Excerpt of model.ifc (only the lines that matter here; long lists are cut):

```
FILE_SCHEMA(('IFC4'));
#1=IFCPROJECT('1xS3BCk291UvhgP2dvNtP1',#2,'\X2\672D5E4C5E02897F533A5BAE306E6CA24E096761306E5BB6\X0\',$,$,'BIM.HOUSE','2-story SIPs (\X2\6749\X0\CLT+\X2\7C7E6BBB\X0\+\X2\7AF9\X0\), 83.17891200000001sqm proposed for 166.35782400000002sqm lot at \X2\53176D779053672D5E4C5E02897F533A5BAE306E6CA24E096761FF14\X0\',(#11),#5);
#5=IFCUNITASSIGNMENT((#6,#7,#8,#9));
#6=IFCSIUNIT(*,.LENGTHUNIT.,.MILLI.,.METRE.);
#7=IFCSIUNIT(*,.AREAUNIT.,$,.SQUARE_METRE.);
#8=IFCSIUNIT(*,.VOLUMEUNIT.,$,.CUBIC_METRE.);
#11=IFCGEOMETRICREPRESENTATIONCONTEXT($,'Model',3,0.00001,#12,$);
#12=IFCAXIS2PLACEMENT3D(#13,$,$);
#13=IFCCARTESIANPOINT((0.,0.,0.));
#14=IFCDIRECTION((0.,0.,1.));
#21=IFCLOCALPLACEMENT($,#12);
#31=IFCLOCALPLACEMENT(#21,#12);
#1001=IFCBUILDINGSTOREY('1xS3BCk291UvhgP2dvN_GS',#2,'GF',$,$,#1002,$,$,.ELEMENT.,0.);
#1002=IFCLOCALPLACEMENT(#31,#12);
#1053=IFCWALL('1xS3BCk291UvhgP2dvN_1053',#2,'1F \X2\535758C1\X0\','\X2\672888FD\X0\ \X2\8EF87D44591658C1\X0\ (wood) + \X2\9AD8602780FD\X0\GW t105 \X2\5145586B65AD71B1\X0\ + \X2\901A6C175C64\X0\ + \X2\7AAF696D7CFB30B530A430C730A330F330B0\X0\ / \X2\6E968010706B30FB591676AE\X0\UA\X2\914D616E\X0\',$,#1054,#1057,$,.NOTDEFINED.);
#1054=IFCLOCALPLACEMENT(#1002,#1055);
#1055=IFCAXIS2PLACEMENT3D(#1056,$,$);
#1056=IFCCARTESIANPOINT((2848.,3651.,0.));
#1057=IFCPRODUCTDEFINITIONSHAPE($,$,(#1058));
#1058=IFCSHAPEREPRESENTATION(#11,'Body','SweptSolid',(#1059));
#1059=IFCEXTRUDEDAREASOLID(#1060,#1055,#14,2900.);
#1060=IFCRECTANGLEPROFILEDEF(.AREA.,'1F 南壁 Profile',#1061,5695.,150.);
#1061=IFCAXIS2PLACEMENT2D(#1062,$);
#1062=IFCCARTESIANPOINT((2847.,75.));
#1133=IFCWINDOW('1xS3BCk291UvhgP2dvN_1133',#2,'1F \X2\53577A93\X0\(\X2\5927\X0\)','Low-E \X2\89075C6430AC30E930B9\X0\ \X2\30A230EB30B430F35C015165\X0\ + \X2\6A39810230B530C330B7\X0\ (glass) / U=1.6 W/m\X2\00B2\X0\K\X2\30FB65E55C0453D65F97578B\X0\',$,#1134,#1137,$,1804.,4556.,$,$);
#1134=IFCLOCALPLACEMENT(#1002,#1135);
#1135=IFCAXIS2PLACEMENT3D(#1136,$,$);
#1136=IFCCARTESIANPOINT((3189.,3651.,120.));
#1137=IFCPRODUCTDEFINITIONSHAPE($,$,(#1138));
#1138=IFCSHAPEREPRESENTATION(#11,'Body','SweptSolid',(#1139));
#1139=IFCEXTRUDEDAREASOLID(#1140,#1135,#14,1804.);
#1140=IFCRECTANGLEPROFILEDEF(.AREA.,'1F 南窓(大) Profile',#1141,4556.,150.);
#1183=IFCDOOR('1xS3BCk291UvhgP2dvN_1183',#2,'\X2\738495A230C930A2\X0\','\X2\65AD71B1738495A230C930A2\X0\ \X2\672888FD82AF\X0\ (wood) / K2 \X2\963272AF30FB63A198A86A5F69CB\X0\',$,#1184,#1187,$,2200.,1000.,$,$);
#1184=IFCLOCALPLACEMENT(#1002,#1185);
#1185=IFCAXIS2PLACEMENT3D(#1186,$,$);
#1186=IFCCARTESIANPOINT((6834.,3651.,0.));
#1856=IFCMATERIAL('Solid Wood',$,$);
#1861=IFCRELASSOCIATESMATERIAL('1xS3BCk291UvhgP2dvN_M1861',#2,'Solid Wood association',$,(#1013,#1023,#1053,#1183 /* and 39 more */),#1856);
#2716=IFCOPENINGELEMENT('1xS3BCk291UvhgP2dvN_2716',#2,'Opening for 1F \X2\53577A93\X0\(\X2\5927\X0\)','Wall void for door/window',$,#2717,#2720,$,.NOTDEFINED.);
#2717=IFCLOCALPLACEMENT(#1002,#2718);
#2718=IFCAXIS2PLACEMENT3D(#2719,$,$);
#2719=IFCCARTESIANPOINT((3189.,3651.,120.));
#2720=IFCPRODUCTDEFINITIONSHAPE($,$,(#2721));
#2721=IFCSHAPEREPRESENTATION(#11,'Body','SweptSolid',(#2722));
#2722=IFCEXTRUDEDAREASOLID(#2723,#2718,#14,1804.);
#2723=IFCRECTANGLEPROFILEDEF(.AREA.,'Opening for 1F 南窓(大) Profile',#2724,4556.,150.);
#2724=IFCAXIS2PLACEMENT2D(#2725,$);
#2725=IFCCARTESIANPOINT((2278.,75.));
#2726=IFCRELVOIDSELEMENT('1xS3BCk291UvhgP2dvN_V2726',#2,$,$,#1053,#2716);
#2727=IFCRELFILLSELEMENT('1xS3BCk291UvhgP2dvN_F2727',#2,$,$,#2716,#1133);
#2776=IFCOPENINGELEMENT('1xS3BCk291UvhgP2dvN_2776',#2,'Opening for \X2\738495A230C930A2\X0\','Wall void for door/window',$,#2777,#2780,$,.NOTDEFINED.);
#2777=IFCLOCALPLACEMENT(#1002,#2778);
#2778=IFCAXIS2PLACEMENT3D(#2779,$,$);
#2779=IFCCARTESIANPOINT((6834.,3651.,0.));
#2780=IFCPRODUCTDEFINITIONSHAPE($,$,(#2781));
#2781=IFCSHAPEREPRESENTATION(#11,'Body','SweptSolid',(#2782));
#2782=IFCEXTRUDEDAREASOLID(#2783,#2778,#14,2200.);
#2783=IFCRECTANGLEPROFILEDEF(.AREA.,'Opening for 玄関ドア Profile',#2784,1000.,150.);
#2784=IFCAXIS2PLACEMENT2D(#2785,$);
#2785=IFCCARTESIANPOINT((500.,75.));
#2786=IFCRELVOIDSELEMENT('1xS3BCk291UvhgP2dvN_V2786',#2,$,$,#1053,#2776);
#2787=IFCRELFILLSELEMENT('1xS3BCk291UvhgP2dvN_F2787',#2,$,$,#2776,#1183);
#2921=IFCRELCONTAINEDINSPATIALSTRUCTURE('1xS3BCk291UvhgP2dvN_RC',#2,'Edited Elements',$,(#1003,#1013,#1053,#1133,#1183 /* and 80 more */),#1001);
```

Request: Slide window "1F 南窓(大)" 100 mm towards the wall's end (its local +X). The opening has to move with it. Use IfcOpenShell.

```python
import ifcopenshell
import ifcopenshell.api.geometry
import ifcopenshell.util.placement
import ifcopenshell.util.unit

model = ifcopenshell.open("model.ifc")
unit_scale = ifcopenshell.util.unit.calculate_unit_scale(model)

window = model.by_guid("1xS3BCk291UvhgP2dvN_1133")
opening = window.FillsVoids[0].RelatingOpeningElement
wall = opening.VoidsElements[0].RelatingBuildingElement

wall_matrix = ifcopenshell.util.placement.get_local_placement(wall.ObjectPlacement)
shift = wall_matrix[:3, 0] * 0.1 / unit_scale
before = ifcopenshell.util.placement.get_local_placement(window.ObjectPlacement)[:3, 3].copy()

# The window is not placed relative to its opening, so move both.
for product in (opening, window):
    matrix = ifcopenshell.util.placement.get_local_placement(product.ObjectPlacement)
    matrix[:3, 3] += shift
    ifcopenshell.api.geometry.edit_object_placement(model, product=product, matrix=matrix, is_si=False)

after = ifcopenshell.util.placement.get_local_placement(window.ObjectPlacement)[:3, 3]
print("window moved by", (after - before).round(3) + 0.0)

model.write("model_rev.ifc")
```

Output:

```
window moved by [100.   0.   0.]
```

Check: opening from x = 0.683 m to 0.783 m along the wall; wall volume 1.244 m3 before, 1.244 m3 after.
